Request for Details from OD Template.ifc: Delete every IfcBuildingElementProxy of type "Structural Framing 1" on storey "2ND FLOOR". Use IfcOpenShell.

First a look at what the model holds.

```python
import ifcopenshell
import ifcopenshell.util.element

model = ifcopenshell.open("Details from OD Template.ifc")
print(model.schema)
storey = next(s for s in model.by_type("IfcBuildingStorey") if s.Name == "2ND FLOOR")
proxies = [e for e in ifcopenshell.util.element.get_decomposition(storey) if e.is_a("IfcBuildingElementProxy")]
seen = {}
for e in proxies:
    element_type = ifcopenshell.util.element.get_type(e)
    name = element_type.Name if element_type not in (None, e) else None
    seen[name] = seen.get(name, 0) + 1
for name, count in sorted(seen.items(), key=str):
    print(count, "x", name)
```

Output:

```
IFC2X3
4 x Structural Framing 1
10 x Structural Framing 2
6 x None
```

```python
import ifcopenshell
import ifcopenshell.api.root
import ifcopenshell.util.element

model = ifcopenshell.open("Details from OD Template.ifc")

storey = next(s for s in model.by_type("IfcBuildingStorey") if s.Name == "2ND FLOOR")
proxies = [e for e in ifcopenshell.util.element.get_decomposition(storey) if e.is_a("IfcBuildingElementProxy")]
targets = [e for e in proxies if (t := ifcopenshell.util.element.get_type(e)) not in (None, e) and t.Name == "Structural Framing 1"]

for e in targets:
    ifcopenshell.api.root.remove_product(model, product=e)
print(len(targets), "removed")

model.write("Details from OD Template_v2.ifc")
```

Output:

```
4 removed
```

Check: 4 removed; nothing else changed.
